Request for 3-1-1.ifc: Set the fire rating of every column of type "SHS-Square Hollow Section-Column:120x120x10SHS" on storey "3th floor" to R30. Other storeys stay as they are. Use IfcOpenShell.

First a look at what the model holds.

```python
import ifcopenshell
import ifcopenshell.util.element

model = ifcopenshell.open("3-1-1.ifc")
print(model.schema)
storey = next(s for s in model.by_type("IfcBuildingStorey") if s.Name == "3th floor")
columns = [e for e in ifcopenshell.util.element.get_decomposition(storey) if e.is_a("IfcColumn")]
seen = {}
for e in columns:
    element_type = ifcopenshell.util.element.get_type(e)
    key = (element_type.Name if element_type != e and element_type else None, ifcopenshell.util.element.get_pset(e, "Pset_ColumnCommon", "FireRating"))
    seen[key] = seen.get(key, 0) + 1
for (name, value), count in sorted(seen.items(), key=str):
    print(count, "x", name, "|", value)
```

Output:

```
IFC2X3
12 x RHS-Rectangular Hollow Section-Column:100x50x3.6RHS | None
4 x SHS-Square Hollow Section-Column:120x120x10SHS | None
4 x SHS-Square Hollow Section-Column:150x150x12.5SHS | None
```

```python
import ifcopenshell
import ifcopenshell.api.pset
import ifcopenshell.util.element

model = ifcopenshell.open("3-1-1.ifc")

storey = next(s for s in model.by_type("IfcBuildingStorey") if s.Name == "3th floor")
columns = [e for e in ifcopenshell.util.element.get_decomposition(storey) if e.is_a("IfcColumn")]

count = 0
for e in columns:
    element_type = ifcopenshell.util.element.get_type(e)
    if element_type in (None, e) or element_type.Name != "SHS-Square Hollow Section-Column:120x120x10SHS":
        continue
    # add_pset returns the element's existing set when there is one.
    pset = ifcopenshell.api.pset.add_pset(model, product=e, name="Pset_ColumnCommon")
    ifcopenshell.api.pset.edit_pset(model, pset=pset, properties={"FireRating": "R30"})
    count += 1

print(count, "columns updated")

model.write("3-1-1_v2.ifc")
```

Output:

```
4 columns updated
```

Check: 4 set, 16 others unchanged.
